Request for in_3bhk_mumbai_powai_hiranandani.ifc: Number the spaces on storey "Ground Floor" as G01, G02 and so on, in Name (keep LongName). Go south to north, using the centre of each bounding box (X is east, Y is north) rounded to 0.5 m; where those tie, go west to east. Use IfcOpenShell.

First a look at what the model holds.

```python
import ifcopenshell
import ifcopenshell.util.element
import ifcopenshell.util.placement

model = ifcopenshell.open("in_3bhk_mumbai_powai_hiranandani.ifc")
print(model.schema)
storey = next(s for s in model.by_type("IfcBuildingStorey") if s.Name == "Ground Floor")
spaces = [e for e in ifcopenshell.util.element.get_decomposition(storey) if e.is_a("IfcSpace")]
for e in sorted(spaces, key=lambda e: e.id()):
    origin = ifcopenshell.util.placement.get_local_placement(e.ObjectPlacement)[:3, 3]
    print(e.id(), e.Name, e.LongName, origin.round(2) + 0.0, sep=" | ")
```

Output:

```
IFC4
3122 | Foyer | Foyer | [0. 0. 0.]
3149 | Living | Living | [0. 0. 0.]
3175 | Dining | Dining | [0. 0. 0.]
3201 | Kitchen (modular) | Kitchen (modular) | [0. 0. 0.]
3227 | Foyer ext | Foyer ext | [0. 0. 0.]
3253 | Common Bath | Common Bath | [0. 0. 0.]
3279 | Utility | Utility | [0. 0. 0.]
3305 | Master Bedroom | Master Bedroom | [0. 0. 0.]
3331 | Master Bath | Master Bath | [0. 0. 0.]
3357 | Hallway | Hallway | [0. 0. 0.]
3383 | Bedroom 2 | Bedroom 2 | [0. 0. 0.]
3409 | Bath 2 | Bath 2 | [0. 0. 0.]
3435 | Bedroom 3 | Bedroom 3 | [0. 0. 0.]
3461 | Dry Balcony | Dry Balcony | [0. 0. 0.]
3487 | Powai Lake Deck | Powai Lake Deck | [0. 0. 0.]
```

```python
import ifcopenshell
import ifcopenshell.geom
import ifcopenshell.util.element
import ifcopenshell.util.shape

model = ifcopenshell.open("in_3bhk_mumbai_powai_hiranandani.ifc")
settings = ifcopenshell.geom.settings()
settings.set("use-world-coords", True)


def centre(element):
    shape = ifcopenshell.geom.create_shape(settings, element)
    return ifcopenshell.util.shape.get_bbox_centroid(shape.geometry)


storey = next(s for s in model.by_type("IfcBuildingStorey") if s.Name == "Ground Floor")
spaces = [e for e in ifcopenshell.util.element.get_decomposition(storey) if e.is_a("IfcSpace")]

# Insertion points can sit at a corner or the storey origin, so sort by the geometry (in metres).
centres = {e: centre(e) for e in spaces}
spaces.sort(key=lambda e: (round(centres[e][1] / 0.5), centres[e][0]))

for i, e in enumerate(spaces, start=1):
    number = f"G{i:02d}"
    e.Name = number
    print(e.id(), number)

model.write("in_3bhk_mumbai_powai_hiranandani_updated.ifc")
```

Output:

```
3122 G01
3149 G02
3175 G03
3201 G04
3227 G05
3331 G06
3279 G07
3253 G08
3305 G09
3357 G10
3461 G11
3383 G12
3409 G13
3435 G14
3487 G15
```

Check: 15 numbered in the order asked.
